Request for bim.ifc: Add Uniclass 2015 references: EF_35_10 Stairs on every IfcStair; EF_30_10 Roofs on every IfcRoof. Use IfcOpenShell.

First a look at what the model holds.

```python
import ifcopenshell

model = ifcopenshell.open("bim.ifc")
print(model.schema)
print("classifications:", [c.Name for c in model.by_type("IfcClassification")])
for ifc_class in ("IfcDoor", "IfcRoof", "IfcStair", "IfcWall", "IfcWindow"):
    print(ifc_class, len(model.by_type(ifc_class)))
```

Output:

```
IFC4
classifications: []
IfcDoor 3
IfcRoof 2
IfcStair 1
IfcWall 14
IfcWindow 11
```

```python
import ifcopenshell
import ifcopenshell.api.classification

model = ifcopenshell.open("bim.ifc")

system = ifcopenshell.api.classification.add_classification(model, classification="Uniclass 2015")

codes = {
    "IfcStair": ("EF_35_10", "Stairs"),
    "IfcRoof": ("EF_30_10", "Roofs"),
}
for ifc_class, (code, name) in codes.items():
    products = model.by_type(ifc_class)
    ifcopenshell.api.classification.add_reference(
        model, products=products, classification=system, identification=code, name=name
    )
    print(code, len(products))

model.write("bim_edited.ifc")
```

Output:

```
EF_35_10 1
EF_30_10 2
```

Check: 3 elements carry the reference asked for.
